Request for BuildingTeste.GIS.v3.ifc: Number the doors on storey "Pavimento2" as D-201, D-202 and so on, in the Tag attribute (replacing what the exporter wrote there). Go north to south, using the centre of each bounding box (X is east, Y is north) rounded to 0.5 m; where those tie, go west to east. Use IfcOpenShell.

First a look at what the model holds.

```python
import ifcopenshell
import ifcopenshell.util.element
import ifcopenshell.util.placement

model = ifcopenshell.open("BuildingTeste.GIS.v3.ifc")
print(model.schema)
storey = next(s for s in model.by_type("IfcBuildingStorey") if s.Name == "Pavimento2")
doors = [e for e in ifcopenshell.util.element.get_decomposition(storey) if e.is_a("IfcDoor")]
for e in sorted(doors, key=lambda e: e.id()):
    origin = ifcopenshell.util.placement.get_local_placement(e.ObjectPlacement)[:3, 3]
    print(e.id(), e.Tag, e.Name, origin.round(2) + 0.0, sep=" | ")
```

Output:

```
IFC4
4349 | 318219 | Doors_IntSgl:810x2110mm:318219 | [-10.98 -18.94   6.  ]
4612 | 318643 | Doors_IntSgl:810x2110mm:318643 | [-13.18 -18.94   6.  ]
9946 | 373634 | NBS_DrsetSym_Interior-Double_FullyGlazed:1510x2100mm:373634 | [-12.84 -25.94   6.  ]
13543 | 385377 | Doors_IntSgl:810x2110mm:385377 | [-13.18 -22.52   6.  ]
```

```python
import ifcopenshell
import ifcopenshell.geom
import ifcopenshell.util.element
import ifcopenshell.util.shape

model = ifcopenshell.open("BuildingTeste.GIS.v3.ifc")
settings = ifcopenshell.geom.settings()
settings.set("use-world-coords", True)


def centre(element):
    shape = ifcopenshell.geom.create_shape(settings, element)
    return ifcopenshell.util.shape.get_bbox_centroid(shape.geometry)


storey = next(s for s in model.by_type("IfcBuildingStorey") if s.Name == "Pavimento2")
doors = [e for e in ifcopenshell.util.element.get_decomposition(storey) if e.is_a("IfcDoor")]

# Insertion points can sit at a corner or the storey origin, so sort by the geometry (in metres).
centres = {e: centre(e) for e in doors}
doors.sort(key=lambda e: (-round(centres[e][1] / 0.5), centres[e][0]))

for i, e in enumerate(doors, start=1):
    number = f"D-2{i:02d}"
    e.Tag = number
    print(e.id(), number)

model.write("BuildingTeste.GIS.v3_rev.ifc")
```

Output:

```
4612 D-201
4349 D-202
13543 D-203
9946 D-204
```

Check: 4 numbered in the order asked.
